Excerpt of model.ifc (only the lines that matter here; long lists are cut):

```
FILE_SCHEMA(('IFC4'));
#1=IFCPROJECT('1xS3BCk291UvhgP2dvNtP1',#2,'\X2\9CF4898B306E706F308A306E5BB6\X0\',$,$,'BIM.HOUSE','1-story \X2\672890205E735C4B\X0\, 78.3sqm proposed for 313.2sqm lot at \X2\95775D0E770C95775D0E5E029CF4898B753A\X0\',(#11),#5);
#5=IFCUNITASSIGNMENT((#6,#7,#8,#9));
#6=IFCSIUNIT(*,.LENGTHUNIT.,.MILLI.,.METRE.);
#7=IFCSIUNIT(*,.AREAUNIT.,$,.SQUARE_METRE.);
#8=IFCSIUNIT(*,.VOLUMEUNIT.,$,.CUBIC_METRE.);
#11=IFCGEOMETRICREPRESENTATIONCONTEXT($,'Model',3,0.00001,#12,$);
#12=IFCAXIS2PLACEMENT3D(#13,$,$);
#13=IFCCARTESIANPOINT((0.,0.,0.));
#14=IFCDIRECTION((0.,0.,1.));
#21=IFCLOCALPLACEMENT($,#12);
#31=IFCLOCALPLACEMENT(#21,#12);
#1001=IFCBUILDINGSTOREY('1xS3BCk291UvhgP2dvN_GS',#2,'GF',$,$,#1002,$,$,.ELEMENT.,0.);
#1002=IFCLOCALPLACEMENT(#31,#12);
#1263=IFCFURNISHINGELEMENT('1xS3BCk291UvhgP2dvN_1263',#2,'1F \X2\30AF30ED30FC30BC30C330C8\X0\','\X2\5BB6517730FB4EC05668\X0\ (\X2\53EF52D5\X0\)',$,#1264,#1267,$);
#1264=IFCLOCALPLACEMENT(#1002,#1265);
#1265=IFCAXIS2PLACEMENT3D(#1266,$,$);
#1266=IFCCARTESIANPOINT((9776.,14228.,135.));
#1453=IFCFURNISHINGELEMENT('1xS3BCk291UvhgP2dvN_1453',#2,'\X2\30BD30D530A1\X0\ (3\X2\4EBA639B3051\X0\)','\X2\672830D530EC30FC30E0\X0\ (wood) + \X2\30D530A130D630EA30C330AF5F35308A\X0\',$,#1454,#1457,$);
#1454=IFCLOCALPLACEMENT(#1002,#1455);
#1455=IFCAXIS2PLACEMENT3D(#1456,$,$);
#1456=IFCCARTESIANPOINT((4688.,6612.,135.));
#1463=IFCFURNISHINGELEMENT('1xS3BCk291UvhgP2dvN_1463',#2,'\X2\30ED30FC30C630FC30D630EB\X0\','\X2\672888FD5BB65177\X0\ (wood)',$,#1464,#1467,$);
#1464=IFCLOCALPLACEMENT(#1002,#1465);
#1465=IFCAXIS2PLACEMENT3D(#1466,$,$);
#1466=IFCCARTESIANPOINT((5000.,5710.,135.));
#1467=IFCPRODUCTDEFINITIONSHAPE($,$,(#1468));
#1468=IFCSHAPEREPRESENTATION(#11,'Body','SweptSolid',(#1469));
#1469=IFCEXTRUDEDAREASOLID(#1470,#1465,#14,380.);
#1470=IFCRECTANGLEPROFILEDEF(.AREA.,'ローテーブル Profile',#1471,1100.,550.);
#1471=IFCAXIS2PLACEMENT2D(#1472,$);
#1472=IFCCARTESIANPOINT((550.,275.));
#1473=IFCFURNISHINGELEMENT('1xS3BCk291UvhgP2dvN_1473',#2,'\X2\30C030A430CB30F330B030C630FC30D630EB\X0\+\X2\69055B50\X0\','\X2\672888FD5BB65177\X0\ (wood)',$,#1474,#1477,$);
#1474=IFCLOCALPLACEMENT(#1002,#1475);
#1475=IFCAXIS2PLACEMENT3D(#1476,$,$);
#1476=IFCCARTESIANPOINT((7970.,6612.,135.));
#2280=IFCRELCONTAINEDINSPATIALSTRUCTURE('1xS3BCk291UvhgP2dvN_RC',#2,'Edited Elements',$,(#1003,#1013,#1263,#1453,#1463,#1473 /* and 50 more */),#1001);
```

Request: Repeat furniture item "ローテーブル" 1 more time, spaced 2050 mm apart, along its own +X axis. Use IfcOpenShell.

```python
import ifcopenshell
import ifcopenshell.api.geometry
import ifcopenshell.api.root
import ifcopenshell.util.element
import ifcopenshell.util.placement
import ifcopenshell.util.unit

model = ifcopenshell.open("model.ifc")
unit_scale = ifcopenshell.util.unit.calculate_unit_scale(model)


def reuse_history(source, copy):
    """copy_class also copies each property set's owner history, people and application; keep the originals."""
    for rel in copy.IsDefinedBy:
        if rel.is_a("IfcRelDefinesByProperties") and (history := rel.RelatingPropertyDefinition.OwnerHistory):
            rel.RelatingPropertyDefinition.OwnerHistory = source.OwnerHistory
            ifcopenshell.util.element.remove_deep2(model, history)


source = model.by_guid("1xS3BCk291UvhgP2dvN_1463")
base = ifcopenshell.util.placement.get_local_placement(source.ObjectPlacement)
step = base[:3, 0] * 2.05 / unit_scale

for i in range(1, 2):
    copy = ifcopenshell.api.root.copy_class(model, product=source)
    copy.Representation = ifcopenshell.util.element.copy_deep(
        model, source.Representation, exclude=["IfcGeometricRepresentationContext", "IfcRepresentationMap"]
    )
    reuse_history(source, copy)
    matrix = base.copy()
    matrix[:3, 3] += i * step
    print("added at", matrix[:3, 3].round(3) + 0.0)
    ifcopenshell.api.geometry.edit_object_placement(model, product=copy, matrix=matrix, is_si=False)

model.write("model_v2.ifc")
```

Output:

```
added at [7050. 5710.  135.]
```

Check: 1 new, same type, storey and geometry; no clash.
